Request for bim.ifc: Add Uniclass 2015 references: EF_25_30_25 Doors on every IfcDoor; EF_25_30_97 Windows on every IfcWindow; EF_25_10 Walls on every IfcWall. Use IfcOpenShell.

First a look at what the model holds.

```python
import ifcopenshell

model = ifcopenshell.open("bim.ifc")
print(model.schema)
print("classifications:", [c.Name for c in model.by_type("IfcClassification")])
for ifc_class in ("IfcDoor", "IfcRoof", "IfcStair", "IfcWall", "IfcWindow"):
    print(ifc_class, len(model.by_type(ifc_class)))
```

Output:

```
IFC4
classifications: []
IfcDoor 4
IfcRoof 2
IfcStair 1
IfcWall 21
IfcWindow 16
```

```python
import ifcopenshell
import ifcopenshell.api.classification

model = ifcopenshell.open("bim.ifc")

system = ifcopenshell.api.classification.add_classification(model, classification="Uniclass 2015")

codes = {
    "IfcDoor": ("EF_25_30_25", "Doors"),
    "IfcWindow": ("EF_25_30_97", "Windows"),
    "IfcWall": ("EF_25_10", "Walls"),
}
for ifc_class, (code, name) in codes.items():
    products = model.by_type(ifc_class)
    ifcopenshell.api.classification.add_reference(
        model, products=products, classification=system, identification=code, name=name
    )
    print(code, len(products))

model.write("bim_v2.ifc")
```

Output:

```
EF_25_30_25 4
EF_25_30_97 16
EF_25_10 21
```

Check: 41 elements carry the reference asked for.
